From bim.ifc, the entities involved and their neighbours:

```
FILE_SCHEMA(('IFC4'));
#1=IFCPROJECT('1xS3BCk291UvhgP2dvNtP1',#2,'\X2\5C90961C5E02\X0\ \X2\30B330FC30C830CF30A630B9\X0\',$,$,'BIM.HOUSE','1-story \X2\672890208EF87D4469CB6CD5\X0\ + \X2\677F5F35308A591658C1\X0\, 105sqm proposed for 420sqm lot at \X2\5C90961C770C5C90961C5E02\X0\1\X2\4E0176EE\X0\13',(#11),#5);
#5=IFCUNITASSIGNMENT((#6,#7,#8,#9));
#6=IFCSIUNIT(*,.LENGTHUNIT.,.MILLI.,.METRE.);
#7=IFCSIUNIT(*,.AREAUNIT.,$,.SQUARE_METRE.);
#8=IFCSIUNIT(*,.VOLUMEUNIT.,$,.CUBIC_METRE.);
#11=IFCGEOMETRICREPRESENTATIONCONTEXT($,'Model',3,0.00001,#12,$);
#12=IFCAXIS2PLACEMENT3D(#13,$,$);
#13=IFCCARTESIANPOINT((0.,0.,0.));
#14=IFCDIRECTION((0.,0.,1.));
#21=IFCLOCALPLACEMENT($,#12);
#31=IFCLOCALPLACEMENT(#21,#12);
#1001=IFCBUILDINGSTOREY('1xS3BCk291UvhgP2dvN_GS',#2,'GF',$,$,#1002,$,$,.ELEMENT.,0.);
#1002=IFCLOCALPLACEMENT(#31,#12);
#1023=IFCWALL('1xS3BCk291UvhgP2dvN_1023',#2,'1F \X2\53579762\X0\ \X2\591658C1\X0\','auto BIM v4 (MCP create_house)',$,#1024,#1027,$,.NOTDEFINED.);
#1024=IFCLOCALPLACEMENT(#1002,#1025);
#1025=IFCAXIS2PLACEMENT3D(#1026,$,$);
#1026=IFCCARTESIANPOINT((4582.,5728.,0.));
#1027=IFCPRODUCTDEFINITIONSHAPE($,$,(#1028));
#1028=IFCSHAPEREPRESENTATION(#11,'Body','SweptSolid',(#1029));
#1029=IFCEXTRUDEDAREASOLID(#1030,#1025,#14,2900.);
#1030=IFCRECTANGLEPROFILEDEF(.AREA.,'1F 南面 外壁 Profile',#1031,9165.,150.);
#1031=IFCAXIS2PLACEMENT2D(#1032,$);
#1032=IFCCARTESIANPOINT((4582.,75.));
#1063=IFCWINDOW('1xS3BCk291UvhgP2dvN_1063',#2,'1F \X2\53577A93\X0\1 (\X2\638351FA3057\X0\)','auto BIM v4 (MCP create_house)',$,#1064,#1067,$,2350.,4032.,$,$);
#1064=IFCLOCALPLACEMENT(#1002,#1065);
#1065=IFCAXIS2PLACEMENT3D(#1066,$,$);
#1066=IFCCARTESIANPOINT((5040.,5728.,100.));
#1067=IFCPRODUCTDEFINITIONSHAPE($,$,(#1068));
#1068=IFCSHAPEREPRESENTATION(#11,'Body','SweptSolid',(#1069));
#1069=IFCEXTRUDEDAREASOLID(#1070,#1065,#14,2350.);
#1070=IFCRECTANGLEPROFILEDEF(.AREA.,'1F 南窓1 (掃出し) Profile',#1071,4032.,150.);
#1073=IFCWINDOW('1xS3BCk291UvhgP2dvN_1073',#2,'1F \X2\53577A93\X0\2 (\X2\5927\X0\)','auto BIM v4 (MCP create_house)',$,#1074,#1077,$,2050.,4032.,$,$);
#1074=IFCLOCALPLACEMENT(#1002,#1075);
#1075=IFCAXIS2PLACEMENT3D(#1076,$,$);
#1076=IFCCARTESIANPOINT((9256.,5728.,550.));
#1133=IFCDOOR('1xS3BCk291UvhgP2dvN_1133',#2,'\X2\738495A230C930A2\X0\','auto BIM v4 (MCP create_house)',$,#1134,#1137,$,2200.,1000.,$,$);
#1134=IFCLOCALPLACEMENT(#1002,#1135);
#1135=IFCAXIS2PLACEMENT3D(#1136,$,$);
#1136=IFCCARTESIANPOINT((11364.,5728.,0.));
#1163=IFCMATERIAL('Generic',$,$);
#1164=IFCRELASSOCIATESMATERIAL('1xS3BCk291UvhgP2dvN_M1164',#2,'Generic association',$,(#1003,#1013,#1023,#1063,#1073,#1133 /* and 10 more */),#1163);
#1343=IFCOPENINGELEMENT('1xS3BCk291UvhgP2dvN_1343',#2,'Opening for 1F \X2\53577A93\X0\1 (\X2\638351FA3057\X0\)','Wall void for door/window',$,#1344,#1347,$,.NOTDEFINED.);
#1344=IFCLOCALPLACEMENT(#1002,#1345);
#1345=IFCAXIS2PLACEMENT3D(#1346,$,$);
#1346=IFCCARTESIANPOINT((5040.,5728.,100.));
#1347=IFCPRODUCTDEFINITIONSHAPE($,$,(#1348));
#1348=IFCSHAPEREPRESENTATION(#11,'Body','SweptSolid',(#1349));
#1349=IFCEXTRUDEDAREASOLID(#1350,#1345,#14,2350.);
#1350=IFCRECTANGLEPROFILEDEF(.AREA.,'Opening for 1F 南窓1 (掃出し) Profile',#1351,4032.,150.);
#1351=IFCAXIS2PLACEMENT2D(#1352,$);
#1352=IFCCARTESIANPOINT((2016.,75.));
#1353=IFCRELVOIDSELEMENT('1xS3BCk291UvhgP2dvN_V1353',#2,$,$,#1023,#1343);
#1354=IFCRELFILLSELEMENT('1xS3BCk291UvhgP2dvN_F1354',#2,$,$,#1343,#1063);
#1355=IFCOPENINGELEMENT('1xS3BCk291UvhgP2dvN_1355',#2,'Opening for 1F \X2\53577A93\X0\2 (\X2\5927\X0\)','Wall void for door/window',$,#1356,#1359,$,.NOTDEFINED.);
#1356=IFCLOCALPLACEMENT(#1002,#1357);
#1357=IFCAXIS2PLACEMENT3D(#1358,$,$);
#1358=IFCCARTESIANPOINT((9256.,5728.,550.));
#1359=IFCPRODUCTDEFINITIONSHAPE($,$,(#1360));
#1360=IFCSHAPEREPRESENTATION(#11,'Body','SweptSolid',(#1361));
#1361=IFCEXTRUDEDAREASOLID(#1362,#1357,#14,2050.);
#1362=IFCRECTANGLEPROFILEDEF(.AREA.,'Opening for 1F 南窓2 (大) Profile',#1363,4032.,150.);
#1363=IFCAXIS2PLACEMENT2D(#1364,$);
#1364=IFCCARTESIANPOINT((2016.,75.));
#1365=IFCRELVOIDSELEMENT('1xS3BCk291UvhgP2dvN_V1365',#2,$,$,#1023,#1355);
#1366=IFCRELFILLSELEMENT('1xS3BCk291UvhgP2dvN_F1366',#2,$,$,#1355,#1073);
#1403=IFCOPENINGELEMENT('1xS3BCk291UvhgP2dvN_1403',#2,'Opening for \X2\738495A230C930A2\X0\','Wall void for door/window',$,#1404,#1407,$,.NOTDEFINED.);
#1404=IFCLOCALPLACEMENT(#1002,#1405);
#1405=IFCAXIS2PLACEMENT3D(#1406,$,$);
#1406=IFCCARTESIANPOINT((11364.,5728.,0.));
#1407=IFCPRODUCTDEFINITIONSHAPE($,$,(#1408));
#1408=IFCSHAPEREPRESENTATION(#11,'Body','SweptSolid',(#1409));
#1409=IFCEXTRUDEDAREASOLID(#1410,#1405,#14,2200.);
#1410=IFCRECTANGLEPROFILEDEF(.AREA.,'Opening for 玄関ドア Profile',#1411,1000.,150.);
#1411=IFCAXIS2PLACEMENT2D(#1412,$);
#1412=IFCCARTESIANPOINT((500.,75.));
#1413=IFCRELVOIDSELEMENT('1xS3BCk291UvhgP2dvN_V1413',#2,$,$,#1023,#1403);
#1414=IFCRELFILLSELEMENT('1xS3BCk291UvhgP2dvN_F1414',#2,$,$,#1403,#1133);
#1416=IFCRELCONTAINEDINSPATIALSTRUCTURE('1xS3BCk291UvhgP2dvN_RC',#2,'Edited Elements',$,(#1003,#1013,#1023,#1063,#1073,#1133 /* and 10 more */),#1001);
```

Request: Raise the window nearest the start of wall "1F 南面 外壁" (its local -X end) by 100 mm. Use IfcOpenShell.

```python
import numpy as np
import ifcopenshell
import ifcopenshell.api.geometry
import ifcopenshell.util.placement
import ifcopenshell.util.unit

model = ifcopenshell.open("bim.ifc")
unit_scale = ifcopenshell.util.unit.calculate_unit_scale(model)

window = model.by_id(1063)
opening = window.FillsVoids[0].RelatingOpeningElement
dz = 0.1 / unit_scale

shift = np.array([0.0, 0.0, dz])
# The window is not placed relative to its opening, so move both.
for product in (opening, window):
    matrix = ifcopenshell.util.placement.get_local_placement(product.ObjectPlacement)
    matrix[:3, 3] += shift
    ifcopenshell.api.geometry.edit_object_placement(model, product=product, matrix=matrix, is_si=False)

print(f"moved by {dz * unit_scale:+.3f} m")

model.write("bim_rev.ifc")
```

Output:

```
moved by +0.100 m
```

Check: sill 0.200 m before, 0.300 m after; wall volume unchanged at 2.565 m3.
